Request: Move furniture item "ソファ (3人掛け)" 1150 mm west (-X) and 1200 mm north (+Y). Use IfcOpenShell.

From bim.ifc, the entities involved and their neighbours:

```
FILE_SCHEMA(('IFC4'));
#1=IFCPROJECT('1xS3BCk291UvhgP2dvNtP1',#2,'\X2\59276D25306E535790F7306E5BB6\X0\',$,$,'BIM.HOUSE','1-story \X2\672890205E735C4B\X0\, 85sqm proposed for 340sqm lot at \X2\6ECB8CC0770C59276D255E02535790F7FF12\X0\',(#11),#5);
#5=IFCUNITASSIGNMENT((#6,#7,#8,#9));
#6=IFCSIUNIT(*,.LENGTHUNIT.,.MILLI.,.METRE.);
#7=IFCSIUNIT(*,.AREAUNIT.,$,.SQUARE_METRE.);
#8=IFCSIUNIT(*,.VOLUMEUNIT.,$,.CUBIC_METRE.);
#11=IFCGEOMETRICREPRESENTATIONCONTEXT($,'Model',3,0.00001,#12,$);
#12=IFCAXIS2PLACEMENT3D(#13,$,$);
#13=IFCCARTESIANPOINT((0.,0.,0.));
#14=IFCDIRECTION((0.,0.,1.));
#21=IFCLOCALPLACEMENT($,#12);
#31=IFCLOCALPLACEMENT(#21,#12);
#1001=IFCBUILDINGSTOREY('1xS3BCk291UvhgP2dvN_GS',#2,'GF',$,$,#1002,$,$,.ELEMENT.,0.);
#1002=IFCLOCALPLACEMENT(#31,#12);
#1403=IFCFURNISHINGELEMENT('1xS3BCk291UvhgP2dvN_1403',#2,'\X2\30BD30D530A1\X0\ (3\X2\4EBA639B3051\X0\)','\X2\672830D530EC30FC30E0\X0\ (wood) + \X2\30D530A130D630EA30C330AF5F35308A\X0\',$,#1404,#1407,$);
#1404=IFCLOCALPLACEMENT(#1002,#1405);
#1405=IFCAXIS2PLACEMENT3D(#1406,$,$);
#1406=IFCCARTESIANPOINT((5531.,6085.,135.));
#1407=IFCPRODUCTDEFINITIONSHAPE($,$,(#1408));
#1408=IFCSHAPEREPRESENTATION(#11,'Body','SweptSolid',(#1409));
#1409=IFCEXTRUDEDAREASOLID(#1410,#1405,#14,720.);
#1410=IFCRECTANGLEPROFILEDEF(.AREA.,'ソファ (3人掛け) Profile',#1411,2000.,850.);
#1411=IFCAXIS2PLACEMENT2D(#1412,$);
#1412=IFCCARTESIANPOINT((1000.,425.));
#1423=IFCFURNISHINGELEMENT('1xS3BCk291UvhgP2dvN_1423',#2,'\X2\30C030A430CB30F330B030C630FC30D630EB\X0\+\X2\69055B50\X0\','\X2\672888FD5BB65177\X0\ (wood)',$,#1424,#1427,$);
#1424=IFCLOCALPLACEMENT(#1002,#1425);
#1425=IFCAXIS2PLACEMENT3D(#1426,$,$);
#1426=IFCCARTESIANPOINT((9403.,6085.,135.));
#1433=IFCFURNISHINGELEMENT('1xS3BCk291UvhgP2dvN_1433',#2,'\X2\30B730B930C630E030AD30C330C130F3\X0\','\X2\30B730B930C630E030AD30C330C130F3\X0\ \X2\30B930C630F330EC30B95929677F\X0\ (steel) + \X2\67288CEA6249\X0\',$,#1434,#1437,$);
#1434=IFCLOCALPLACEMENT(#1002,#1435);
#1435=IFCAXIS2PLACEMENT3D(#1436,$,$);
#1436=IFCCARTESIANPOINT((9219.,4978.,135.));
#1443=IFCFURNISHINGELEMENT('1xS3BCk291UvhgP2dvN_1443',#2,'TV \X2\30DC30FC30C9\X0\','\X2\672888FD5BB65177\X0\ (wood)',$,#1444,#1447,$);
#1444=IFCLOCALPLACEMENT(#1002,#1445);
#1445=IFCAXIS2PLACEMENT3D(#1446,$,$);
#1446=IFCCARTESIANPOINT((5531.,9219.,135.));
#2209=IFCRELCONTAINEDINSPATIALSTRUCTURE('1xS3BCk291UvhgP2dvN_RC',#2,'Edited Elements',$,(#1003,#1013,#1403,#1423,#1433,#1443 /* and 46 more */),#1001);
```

```python
import ifcopenshell
import ifcopenshell.api.geometry
import ifcopenshell.util.placement

model = ifcopenshell.open("bim.ifc")

item = model.by_id(1403)
matrix = ifcopenshell.util.placement.get_local_placement(item.ObjectPlacement)
matrix[0, 3] -= 1150.0
matrix[1, 3] += 1200.0
ifcopenshell.api.geometry.edit_object_placement(model, product=item, matrix=matrix, is_si=False)

print(ifcopenshell.util.placement.get_local_placement(item.ObjectPlacement).round(3) + 0.0)

model.write("bim-out.ifc")
```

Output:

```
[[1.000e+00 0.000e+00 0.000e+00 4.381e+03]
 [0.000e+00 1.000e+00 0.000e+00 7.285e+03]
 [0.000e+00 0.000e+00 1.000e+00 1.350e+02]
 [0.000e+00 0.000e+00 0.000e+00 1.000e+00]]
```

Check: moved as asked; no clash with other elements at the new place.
